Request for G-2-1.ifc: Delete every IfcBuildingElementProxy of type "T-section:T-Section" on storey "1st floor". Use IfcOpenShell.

First a look at what the model holds.

```python
import ifcopenshell
import ifcopenshell.util.element

model = ifcopenshell.open("G-2-1.ifc")
print(model.schema)
storey = next(s for s in model.by_type("IfcBuildingStorey") if s.Name == "1st floor")
proxies = [e for e in ifcopenshell.util.element.get_decomposition(storey) if e.is_a("IfcBuildingElementProxy")]
seen = {}
for e in proxies:
    element_type = ifcopenshell.util.element.get_type(e)
    name = element_type.Name if element_type not in (None, e) else None
    seen[name] = seen.get(name, 0) + 1
for name, count in sorted(seen.items(), key=str):
    print(count, "x", name)
```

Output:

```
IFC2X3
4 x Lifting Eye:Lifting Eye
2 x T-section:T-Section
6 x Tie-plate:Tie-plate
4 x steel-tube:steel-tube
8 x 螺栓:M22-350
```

```python
import ifcopenshell
import ifcopenshell.api.root
import ifcopenshell.util.element

model = ifcopenshell.open("G-2-1.ifc")

storey = next(s for s in model.by_type("IfcBuildingStorey") if s.Name == "1st floor")
proxies = [e for e in ifcopenshell.util.element.get_decomposition(storey) if e.is_a("IfcBuildingElementProxy")]
targets = [e for e in proxies if (t := ifcopenshell.util.element.get_type(e)) not in (None, e) and t.Name == "T-section:T-Section"]

for e in targets:
    ifcopenshell.api.root.remove_product(model, product=e)
print(len(targets), "removed")

model.write("G-2-1_rev.ifc")
```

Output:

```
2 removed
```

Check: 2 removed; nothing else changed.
